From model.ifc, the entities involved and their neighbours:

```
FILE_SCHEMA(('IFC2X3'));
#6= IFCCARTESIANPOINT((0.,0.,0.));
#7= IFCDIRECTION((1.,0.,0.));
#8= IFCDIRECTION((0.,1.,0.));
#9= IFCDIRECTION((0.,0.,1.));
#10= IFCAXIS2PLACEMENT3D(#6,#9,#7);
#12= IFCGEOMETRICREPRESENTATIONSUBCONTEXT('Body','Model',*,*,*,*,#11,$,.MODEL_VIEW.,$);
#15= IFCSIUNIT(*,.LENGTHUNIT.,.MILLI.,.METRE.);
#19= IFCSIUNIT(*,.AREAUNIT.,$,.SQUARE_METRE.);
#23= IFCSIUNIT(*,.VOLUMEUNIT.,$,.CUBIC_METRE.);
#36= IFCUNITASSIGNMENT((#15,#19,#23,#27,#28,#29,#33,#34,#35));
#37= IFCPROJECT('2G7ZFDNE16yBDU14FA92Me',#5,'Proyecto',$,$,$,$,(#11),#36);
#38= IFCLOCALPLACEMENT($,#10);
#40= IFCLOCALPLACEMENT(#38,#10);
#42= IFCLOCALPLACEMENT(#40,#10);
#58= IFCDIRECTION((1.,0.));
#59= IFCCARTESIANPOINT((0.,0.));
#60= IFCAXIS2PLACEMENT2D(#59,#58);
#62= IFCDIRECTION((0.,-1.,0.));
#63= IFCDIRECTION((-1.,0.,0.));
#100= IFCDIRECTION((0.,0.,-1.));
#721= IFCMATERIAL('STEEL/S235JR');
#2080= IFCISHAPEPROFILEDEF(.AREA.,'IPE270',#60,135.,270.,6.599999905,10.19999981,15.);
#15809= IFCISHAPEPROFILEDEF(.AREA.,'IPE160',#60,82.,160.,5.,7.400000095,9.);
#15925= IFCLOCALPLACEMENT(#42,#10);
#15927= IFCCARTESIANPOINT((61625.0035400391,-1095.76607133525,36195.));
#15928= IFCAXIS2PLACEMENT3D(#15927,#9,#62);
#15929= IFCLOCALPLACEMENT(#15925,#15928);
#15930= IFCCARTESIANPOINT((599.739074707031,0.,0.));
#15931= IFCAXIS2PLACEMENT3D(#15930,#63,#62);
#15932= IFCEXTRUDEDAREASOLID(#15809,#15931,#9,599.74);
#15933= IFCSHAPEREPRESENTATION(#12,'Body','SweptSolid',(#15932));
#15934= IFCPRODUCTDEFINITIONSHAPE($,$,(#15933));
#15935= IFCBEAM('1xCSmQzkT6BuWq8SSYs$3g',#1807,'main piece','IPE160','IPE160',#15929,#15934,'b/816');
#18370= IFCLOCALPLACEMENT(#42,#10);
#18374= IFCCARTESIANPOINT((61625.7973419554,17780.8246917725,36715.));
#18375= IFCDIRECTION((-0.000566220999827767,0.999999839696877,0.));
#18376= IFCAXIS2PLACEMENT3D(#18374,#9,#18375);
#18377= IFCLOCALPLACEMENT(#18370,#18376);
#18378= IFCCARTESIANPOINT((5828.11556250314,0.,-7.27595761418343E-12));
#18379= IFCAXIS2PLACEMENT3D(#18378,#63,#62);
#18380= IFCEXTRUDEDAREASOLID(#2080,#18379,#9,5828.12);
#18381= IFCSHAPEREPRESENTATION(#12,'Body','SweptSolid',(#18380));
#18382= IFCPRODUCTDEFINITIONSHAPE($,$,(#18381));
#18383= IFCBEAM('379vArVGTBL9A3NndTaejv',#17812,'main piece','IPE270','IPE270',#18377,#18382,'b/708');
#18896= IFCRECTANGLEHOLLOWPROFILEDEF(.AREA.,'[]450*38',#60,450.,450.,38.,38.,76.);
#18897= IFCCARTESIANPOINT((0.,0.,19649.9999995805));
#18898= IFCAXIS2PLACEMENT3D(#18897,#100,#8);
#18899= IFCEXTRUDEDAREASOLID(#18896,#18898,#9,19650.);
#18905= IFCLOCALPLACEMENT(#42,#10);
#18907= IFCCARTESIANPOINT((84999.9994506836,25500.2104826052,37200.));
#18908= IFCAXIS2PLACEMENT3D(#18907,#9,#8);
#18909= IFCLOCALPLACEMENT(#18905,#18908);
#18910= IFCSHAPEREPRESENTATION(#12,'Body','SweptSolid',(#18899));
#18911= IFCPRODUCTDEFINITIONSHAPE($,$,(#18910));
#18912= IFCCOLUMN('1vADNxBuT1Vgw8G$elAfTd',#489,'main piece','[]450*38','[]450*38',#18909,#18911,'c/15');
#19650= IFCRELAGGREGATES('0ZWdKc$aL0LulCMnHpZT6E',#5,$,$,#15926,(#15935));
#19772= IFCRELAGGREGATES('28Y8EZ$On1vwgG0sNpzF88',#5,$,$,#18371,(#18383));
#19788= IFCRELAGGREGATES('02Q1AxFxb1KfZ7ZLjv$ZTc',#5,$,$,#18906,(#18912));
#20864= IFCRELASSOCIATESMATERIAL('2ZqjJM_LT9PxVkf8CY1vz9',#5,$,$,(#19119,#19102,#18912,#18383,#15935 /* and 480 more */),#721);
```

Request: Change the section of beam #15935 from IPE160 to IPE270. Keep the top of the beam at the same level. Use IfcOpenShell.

```python
import ifcopenshell
import ifcopenshell.util.element
import ifcopenshell.util.representation

model = ifcopenshell.open("model.ifc")

member = model.by_guid("1xCSmQzkT6BuWq8SSYs$3g")
source = next(p for p in model.by_type("IfcIShapeProfileDef") if p.ProfileName == "IPE270")

body = ifcopenshell.util.representation.get_representation(member, "Model", "Body")
solid = body.Items[0]
old_profile = solid.SweptArea

# Copy the section's sizes but keep this member's own profile position.
profile = ifcopenshell.util.element.copy(model, source)
# Profiles are centred, so shift by half the change in depth to hold the top.
shift = (old_profile.OverallDepth - profile.OverallDepth) / 2
x, y = old_profile.Position.Location.Coordinates
up = (0.0, 1.0)  # upwards, in the solid's own plane
location = model.createIfcCartesianPoint((x + up[0] * shift, y + up[1] * shift))
profile.Position = model.createIfcAxis2Placement2D(location, old_profile.Position.RefDirection)
solid.SweptArea = profile
if not model.get_total_inverses(old_profile):
    ifcopenshell.util.element.remove_deep2(model, old_profile)
member.Description = member.Description.replace("IPE160", "IPE270")
member.ObjectType = member.ObjectType.replace("IPE160", "IPE270")

print(solid.SweptArea)

model.write("model_updated.ifc")
```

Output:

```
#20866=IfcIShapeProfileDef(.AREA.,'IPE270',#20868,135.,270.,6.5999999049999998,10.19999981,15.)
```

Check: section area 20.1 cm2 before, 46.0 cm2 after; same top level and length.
